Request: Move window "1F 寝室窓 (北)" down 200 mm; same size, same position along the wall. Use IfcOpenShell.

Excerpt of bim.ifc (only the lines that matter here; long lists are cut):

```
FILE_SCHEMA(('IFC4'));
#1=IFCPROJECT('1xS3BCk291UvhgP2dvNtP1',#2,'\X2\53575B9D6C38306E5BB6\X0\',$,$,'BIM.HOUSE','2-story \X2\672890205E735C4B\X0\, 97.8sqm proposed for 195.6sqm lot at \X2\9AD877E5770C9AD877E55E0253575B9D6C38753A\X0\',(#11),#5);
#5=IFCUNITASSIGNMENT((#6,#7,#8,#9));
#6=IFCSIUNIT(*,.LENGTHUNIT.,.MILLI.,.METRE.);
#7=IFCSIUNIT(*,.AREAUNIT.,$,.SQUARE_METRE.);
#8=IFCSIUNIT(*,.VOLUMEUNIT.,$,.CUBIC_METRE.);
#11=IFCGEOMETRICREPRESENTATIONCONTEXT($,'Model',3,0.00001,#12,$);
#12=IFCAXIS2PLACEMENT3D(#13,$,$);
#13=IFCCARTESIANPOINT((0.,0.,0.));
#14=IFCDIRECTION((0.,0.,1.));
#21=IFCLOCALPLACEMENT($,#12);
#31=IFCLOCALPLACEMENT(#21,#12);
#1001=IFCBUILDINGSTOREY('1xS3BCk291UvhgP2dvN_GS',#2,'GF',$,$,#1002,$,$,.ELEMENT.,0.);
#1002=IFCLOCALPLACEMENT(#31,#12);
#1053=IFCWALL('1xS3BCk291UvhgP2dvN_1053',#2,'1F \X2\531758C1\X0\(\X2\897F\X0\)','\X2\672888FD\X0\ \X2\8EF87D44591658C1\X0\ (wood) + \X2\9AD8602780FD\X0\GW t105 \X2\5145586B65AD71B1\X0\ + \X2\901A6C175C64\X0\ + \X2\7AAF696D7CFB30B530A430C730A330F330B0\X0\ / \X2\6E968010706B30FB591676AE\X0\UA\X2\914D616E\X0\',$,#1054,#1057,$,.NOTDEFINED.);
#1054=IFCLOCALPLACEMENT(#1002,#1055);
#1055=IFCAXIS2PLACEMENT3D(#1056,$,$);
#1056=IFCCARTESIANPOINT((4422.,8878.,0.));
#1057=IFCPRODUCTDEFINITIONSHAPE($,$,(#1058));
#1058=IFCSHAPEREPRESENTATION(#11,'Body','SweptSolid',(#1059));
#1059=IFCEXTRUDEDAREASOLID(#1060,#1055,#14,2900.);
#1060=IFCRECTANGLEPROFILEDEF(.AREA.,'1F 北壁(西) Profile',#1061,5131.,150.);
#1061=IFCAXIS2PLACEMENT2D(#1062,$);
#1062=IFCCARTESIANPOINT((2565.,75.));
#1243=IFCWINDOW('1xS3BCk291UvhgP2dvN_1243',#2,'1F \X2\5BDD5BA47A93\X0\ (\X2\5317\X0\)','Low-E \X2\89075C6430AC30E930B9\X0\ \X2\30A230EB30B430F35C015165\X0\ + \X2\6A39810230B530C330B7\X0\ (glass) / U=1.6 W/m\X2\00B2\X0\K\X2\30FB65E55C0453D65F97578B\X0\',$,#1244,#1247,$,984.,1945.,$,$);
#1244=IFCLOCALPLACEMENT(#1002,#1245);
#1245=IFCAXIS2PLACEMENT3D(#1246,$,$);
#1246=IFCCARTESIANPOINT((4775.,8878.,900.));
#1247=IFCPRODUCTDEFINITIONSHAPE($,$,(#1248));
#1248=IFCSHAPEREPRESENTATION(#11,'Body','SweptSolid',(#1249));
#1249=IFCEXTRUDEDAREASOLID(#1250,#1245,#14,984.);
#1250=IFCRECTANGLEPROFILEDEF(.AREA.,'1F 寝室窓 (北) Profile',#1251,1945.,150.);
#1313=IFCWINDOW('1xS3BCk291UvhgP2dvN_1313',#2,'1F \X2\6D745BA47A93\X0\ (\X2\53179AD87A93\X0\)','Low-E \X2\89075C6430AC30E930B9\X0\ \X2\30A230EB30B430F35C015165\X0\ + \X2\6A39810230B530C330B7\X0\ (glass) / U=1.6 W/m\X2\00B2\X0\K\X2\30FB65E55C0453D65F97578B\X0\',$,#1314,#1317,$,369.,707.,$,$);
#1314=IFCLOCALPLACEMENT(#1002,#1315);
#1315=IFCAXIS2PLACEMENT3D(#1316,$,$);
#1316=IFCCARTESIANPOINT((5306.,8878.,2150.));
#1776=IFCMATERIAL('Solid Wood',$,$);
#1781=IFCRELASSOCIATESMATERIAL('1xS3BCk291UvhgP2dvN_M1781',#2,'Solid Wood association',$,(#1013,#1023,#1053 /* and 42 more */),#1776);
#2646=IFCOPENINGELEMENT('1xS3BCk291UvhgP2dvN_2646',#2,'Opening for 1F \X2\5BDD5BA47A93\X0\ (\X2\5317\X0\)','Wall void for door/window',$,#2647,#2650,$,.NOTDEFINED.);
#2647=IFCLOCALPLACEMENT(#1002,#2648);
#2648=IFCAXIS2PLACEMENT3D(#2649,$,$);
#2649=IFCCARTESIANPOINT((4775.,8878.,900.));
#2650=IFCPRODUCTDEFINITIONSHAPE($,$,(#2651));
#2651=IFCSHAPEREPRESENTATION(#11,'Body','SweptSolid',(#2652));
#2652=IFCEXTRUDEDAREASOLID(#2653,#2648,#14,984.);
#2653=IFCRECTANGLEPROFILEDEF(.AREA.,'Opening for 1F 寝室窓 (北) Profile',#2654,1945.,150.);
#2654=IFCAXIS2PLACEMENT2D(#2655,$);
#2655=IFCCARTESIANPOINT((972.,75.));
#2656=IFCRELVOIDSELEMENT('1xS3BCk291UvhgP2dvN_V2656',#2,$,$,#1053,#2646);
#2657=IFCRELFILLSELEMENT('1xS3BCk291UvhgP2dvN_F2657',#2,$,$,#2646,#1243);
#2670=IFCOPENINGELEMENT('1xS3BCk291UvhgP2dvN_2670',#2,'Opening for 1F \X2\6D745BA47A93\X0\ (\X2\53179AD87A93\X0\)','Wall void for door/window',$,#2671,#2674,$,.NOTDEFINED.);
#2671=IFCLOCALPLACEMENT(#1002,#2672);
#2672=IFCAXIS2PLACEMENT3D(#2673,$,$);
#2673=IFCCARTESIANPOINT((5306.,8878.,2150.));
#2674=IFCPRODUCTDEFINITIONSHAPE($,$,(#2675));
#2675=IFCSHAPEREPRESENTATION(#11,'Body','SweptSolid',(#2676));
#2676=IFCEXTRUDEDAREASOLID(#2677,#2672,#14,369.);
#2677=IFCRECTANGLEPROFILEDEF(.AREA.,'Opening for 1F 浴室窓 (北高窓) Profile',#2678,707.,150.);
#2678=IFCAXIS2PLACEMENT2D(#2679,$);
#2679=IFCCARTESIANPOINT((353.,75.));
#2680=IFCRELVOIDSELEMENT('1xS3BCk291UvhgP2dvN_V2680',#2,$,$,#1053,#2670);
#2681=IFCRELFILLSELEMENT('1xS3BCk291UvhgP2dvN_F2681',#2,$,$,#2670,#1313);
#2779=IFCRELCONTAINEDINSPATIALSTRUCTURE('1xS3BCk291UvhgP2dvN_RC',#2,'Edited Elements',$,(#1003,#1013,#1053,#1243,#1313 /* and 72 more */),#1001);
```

```python
import numpy as np
import ifcopenshell
import ifcopenshell.api.geometry
import ifcopenshell.util.placement
import ifcopenshell.util.unit

model = ifcopenshell.open("bim.ifc")
unit_scale = ifcopenshell.util.unit.calculate_unit_scale(model)

window = model.by_id(1243)
opening = window.FillsVoids[0].RelatingOpeningElement
dz = -0.2 / unit_scale

shift = np.array([0.0, 0.0, dz])
# The window is not placed relative to its opening, so move both.
for product in (opening, window):
    matrix = ifcopenshell.util.placement.get_local_placement(product.ObjectPlacement)
    matrix[:3, 3] += shift
    ifcopenshell.api.geometry.edit_object_placement(model, product=product, matrix=matrix, is_si=False)

print(f"moved by {dz * unit_scale:+.3f} m")

model.write("bim-out.ifc")
```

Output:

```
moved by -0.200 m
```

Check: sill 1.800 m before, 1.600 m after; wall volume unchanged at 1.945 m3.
